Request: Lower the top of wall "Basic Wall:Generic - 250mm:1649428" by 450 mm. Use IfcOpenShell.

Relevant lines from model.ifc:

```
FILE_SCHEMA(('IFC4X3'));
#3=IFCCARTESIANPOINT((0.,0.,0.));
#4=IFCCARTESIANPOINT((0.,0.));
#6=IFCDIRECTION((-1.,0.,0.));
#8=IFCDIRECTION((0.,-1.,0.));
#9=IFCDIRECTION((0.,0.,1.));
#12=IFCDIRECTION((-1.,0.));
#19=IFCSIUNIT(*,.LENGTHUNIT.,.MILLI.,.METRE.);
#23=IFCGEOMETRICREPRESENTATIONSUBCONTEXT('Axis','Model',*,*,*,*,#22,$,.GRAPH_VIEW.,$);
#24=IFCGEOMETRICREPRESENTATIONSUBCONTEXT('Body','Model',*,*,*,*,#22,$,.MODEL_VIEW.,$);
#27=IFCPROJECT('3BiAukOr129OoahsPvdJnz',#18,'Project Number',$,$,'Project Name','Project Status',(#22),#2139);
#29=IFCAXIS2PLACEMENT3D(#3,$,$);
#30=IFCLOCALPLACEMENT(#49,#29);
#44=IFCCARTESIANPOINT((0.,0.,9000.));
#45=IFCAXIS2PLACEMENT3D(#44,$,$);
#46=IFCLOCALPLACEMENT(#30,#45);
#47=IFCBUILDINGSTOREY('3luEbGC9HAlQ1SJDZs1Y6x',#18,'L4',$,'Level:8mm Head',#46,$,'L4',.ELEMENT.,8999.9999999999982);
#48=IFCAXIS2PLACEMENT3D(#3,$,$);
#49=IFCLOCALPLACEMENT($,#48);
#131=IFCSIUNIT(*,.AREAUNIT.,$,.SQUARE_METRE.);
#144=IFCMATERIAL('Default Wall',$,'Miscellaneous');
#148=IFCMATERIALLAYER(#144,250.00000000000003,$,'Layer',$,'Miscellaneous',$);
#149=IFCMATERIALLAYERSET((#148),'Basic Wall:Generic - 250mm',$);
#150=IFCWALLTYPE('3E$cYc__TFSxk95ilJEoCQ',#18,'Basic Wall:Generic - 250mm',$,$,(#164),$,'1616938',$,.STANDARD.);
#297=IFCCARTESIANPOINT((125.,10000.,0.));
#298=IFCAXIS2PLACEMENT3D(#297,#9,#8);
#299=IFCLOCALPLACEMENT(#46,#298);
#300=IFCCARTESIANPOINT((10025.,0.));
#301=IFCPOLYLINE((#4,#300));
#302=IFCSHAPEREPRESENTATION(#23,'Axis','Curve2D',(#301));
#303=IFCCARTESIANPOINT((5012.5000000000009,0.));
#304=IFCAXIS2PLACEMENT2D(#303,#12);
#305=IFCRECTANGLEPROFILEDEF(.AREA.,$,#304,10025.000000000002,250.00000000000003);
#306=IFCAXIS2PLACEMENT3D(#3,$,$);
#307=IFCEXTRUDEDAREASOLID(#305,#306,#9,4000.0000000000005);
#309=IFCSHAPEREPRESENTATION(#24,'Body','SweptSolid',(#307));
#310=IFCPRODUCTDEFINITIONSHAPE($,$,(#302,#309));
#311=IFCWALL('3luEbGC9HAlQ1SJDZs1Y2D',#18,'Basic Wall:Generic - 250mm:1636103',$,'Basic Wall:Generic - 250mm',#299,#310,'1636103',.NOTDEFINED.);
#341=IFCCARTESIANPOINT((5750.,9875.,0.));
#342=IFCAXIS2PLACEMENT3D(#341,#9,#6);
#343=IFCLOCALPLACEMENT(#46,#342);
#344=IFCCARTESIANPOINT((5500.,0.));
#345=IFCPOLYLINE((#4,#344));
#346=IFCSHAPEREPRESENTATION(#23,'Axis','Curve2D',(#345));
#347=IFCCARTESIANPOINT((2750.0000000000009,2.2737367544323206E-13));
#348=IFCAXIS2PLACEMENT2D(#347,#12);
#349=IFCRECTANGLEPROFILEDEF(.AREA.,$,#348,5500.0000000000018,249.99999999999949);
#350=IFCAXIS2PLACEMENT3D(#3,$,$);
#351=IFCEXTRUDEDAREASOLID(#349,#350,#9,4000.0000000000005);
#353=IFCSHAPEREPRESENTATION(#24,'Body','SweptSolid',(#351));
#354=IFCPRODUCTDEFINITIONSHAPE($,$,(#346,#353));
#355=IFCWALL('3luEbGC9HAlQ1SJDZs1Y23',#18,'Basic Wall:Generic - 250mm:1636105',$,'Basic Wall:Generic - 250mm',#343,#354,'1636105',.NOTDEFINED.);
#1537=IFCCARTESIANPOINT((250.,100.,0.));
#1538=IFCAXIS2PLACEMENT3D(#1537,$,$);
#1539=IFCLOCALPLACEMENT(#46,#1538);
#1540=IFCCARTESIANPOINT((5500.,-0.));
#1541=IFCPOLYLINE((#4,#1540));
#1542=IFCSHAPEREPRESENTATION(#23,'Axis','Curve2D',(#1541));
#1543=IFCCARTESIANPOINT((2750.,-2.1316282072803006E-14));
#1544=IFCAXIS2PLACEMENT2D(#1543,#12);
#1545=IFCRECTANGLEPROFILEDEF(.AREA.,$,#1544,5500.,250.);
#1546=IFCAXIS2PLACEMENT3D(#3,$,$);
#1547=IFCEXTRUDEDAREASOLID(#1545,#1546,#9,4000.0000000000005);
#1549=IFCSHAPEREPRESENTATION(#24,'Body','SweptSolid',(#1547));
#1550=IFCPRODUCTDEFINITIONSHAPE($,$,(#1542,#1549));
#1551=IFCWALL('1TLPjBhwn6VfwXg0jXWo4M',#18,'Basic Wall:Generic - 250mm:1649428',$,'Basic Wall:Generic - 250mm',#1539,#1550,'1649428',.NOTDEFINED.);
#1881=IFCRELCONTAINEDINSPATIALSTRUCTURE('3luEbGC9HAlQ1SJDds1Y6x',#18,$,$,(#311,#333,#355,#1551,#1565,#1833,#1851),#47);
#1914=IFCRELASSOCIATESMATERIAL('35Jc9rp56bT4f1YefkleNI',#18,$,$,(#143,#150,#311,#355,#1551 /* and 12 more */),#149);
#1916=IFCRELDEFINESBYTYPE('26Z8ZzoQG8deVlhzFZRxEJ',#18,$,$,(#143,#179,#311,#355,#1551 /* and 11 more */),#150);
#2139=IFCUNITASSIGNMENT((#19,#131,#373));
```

```python
import ifcopenshell
import ifcopenshell.geom
import ifcopenshell.util.representation
import ifcopenshell.util.shape
import ifcopenshell.util.unit

model = ifcopenshell.open("model.ifc")
unit_scale = ifcopenshell.util.unit.calculate_unit_scale(model)
settings = ifcopenshell.geom.settings()


def volume(element):
    """Net volume in cubic metres, openings subtracted."""
    shape = ifcopenshell.geom.create_shape(settings, element)
    return ifcopenshell.util.shape.get_volume(shape.geometry)


wall = model.by_guid("1TLPjBhwn6VfwXg0jXWo4M")
before = volume(wall)

body = ifcopenshell.util.representation.get_representation(wall, "Model", "Body")
solid = body.Items[0]
old_height = solid.Depth
solid.Depth -= 0.45 / unit_scale
after = volume(wall)

print(f"height {old_height:g} -> {solid.Depth:g}, volume {before:.3f} -> {after:.3f} m3")

model.write("model_rev.ifc")
```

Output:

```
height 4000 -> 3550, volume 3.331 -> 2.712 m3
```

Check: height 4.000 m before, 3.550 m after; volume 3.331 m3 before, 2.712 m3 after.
